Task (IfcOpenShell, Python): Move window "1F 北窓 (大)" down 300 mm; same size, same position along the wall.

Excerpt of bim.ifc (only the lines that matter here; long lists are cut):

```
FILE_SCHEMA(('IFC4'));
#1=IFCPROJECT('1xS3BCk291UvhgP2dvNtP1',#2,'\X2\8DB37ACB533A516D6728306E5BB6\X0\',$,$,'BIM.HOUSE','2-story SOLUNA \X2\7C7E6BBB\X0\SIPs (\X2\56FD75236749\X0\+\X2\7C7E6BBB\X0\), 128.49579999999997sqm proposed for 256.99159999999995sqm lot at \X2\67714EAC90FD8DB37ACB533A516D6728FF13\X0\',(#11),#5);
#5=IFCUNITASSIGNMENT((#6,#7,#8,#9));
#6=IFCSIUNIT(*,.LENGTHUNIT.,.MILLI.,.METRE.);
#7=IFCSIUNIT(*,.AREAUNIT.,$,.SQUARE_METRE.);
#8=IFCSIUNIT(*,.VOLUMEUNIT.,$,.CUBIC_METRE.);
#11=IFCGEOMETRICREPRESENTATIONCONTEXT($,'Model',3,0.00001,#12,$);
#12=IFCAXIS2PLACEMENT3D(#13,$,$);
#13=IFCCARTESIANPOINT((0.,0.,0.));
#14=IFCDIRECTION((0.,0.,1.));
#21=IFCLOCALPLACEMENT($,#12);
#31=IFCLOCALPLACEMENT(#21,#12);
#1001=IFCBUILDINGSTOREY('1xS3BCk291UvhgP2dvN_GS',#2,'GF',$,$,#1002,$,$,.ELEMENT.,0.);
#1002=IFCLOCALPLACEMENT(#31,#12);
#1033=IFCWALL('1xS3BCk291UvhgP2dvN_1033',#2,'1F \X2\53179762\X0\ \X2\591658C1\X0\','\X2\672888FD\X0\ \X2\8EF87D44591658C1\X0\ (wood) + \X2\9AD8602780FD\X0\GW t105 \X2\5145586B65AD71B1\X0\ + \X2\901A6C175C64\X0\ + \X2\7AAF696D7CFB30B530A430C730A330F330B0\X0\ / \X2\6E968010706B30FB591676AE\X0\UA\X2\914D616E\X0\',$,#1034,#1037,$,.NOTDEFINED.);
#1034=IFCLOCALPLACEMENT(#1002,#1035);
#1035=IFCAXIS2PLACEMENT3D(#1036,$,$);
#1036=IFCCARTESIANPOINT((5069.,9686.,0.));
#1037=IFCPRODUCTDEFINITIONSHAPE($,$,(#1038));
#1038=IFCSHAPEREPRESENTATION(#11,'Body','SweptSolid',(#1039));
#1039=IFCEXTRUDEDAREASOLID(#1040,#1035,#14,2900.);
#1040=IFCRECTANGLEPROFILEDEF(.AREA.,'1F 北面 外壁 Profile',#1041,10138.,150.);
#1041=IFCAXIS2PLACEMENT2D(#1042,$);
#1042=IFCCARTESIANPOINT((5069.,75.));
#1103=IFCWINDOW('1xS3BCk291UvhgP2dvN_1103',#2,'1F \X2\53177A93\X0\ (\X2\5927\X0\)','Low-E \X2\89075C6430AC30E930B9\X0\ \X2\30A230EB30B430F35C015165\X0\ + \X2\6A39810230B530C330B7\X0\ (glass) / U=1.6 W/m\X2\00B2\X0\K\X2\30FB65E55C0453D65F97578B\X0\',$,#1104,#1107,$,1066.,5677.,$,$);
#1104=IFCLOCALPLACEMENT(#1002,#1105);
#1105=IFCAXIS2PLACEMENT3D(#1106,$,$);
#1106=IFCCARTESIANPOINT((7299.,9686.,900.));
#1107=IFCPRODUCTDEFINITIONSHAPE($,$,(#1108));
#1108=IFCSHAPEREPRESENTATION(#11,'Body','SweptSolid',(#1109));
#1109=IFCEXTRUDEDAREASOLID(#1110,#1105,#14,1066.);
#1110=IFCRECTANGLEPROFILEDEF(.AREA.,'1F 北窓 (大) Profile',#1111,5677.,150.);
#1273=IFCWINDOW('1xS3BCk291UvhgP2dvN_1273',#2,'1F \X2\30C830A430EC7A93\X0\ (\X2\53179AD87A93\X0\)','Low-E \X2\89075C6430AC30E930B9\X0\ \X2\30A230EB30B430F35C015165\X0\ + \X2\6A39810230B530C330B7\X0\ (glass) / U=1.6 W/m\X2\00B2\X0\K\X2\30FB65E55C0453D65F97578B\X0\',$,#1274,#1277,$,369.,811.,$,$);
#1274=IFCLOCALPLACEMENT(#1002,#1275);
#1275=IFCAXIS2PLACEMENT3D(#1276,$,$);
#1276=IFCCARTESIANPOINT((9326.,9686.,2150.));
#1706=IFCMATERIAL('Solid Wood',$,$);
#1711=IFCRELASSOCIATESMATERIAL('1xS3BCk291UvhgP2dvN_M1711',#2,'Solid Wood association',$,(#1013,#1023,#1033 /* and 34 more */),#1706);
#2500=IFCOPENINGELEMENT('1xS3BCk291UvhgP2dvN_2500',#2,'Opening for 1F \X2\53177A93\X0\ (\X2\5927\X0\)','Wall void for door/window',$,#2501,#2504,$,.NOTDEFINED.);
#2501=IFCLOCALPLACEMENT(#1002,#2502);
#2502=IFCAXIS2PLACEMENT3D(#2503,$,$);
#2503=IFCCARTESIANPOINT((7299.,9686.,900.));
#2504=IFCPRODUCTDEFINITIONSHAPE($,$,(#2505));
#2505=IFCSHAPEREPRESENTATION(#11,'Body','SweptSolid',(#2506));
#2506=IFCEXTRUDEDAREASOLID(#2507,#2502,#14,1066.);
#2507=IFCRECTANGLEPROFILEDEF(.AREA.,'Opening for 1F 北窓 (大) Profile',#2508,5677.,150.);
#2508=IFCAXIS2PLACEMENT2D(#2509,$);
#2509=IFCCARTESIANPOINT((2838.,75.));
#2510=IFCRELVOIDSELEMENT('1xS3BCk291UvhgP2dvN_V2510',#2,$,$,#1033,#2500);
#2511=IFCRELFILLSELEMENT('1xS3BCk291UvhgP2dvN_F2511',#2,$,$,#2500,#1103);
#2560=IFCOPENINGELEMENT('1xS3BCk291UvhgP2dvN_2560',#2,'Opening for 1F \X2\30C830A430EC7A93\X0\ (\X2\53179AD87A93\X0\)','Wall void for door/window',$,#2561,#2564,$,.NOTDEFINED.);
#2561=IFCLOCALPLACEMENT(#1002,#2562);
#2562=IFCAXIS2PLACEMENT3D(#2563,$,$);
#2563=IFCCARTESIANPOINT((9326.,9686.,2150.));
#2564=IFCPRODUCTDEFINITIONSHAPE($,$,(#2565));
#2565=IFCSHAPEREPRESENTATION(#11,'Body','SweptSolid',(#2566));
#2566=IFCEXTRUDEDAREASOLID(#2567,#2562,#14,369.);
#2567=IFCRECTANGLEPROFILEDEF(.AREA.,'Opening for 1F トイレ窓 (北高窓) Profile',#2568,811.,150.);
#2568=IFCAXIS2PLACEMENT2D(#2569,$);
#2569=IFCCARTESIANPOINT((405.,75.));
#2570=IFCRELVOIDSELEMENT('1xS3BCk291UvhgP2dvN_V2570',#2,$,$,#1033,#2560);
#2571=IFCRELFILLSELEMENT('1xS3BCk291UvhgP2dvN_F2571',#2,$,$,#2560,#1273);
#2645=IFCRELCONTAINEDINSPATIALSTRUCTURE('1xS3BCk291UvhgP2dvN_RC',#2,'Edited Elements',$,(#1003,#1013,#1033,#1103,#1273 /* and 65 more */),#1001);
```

```python
import numpy as np
import ifcopenshell
import ifcopenshell.api.geometry
import ifcopenshell.util.placement
import ifcopenshell.util.unit

model = ifcopenshell.open("bim.ifc")
unit_scale = ifcopenshell.util.unit.calculate_unit_scale(model)

window = model.by_guid("1xS3BCk291UvhgP2dvN_1103")
opening = window.FillsVoids[0].RelatingOpeningElement
dz = -0.3 / unit_scale

shift = np.array([0.0, 0.0, dz])
# The window is not placed relative to its opening, so move both.
for product in (opening, window):
    matrix = ifcopenshell.util.placement.get_local_placement(product.ObjectPlacement)
    matrix[:3, 3] += shift
    ifcopenshell.api.geometry.edit_object_placement(model, product=product, matrix=matrix, is_si=False)

print(f"moved by {dz * unit_scale:+.3f} m")

model.write("bim_v2.ifc")
```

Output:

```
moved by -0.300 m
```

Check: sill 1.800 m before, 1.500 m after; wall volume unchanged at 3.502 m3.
